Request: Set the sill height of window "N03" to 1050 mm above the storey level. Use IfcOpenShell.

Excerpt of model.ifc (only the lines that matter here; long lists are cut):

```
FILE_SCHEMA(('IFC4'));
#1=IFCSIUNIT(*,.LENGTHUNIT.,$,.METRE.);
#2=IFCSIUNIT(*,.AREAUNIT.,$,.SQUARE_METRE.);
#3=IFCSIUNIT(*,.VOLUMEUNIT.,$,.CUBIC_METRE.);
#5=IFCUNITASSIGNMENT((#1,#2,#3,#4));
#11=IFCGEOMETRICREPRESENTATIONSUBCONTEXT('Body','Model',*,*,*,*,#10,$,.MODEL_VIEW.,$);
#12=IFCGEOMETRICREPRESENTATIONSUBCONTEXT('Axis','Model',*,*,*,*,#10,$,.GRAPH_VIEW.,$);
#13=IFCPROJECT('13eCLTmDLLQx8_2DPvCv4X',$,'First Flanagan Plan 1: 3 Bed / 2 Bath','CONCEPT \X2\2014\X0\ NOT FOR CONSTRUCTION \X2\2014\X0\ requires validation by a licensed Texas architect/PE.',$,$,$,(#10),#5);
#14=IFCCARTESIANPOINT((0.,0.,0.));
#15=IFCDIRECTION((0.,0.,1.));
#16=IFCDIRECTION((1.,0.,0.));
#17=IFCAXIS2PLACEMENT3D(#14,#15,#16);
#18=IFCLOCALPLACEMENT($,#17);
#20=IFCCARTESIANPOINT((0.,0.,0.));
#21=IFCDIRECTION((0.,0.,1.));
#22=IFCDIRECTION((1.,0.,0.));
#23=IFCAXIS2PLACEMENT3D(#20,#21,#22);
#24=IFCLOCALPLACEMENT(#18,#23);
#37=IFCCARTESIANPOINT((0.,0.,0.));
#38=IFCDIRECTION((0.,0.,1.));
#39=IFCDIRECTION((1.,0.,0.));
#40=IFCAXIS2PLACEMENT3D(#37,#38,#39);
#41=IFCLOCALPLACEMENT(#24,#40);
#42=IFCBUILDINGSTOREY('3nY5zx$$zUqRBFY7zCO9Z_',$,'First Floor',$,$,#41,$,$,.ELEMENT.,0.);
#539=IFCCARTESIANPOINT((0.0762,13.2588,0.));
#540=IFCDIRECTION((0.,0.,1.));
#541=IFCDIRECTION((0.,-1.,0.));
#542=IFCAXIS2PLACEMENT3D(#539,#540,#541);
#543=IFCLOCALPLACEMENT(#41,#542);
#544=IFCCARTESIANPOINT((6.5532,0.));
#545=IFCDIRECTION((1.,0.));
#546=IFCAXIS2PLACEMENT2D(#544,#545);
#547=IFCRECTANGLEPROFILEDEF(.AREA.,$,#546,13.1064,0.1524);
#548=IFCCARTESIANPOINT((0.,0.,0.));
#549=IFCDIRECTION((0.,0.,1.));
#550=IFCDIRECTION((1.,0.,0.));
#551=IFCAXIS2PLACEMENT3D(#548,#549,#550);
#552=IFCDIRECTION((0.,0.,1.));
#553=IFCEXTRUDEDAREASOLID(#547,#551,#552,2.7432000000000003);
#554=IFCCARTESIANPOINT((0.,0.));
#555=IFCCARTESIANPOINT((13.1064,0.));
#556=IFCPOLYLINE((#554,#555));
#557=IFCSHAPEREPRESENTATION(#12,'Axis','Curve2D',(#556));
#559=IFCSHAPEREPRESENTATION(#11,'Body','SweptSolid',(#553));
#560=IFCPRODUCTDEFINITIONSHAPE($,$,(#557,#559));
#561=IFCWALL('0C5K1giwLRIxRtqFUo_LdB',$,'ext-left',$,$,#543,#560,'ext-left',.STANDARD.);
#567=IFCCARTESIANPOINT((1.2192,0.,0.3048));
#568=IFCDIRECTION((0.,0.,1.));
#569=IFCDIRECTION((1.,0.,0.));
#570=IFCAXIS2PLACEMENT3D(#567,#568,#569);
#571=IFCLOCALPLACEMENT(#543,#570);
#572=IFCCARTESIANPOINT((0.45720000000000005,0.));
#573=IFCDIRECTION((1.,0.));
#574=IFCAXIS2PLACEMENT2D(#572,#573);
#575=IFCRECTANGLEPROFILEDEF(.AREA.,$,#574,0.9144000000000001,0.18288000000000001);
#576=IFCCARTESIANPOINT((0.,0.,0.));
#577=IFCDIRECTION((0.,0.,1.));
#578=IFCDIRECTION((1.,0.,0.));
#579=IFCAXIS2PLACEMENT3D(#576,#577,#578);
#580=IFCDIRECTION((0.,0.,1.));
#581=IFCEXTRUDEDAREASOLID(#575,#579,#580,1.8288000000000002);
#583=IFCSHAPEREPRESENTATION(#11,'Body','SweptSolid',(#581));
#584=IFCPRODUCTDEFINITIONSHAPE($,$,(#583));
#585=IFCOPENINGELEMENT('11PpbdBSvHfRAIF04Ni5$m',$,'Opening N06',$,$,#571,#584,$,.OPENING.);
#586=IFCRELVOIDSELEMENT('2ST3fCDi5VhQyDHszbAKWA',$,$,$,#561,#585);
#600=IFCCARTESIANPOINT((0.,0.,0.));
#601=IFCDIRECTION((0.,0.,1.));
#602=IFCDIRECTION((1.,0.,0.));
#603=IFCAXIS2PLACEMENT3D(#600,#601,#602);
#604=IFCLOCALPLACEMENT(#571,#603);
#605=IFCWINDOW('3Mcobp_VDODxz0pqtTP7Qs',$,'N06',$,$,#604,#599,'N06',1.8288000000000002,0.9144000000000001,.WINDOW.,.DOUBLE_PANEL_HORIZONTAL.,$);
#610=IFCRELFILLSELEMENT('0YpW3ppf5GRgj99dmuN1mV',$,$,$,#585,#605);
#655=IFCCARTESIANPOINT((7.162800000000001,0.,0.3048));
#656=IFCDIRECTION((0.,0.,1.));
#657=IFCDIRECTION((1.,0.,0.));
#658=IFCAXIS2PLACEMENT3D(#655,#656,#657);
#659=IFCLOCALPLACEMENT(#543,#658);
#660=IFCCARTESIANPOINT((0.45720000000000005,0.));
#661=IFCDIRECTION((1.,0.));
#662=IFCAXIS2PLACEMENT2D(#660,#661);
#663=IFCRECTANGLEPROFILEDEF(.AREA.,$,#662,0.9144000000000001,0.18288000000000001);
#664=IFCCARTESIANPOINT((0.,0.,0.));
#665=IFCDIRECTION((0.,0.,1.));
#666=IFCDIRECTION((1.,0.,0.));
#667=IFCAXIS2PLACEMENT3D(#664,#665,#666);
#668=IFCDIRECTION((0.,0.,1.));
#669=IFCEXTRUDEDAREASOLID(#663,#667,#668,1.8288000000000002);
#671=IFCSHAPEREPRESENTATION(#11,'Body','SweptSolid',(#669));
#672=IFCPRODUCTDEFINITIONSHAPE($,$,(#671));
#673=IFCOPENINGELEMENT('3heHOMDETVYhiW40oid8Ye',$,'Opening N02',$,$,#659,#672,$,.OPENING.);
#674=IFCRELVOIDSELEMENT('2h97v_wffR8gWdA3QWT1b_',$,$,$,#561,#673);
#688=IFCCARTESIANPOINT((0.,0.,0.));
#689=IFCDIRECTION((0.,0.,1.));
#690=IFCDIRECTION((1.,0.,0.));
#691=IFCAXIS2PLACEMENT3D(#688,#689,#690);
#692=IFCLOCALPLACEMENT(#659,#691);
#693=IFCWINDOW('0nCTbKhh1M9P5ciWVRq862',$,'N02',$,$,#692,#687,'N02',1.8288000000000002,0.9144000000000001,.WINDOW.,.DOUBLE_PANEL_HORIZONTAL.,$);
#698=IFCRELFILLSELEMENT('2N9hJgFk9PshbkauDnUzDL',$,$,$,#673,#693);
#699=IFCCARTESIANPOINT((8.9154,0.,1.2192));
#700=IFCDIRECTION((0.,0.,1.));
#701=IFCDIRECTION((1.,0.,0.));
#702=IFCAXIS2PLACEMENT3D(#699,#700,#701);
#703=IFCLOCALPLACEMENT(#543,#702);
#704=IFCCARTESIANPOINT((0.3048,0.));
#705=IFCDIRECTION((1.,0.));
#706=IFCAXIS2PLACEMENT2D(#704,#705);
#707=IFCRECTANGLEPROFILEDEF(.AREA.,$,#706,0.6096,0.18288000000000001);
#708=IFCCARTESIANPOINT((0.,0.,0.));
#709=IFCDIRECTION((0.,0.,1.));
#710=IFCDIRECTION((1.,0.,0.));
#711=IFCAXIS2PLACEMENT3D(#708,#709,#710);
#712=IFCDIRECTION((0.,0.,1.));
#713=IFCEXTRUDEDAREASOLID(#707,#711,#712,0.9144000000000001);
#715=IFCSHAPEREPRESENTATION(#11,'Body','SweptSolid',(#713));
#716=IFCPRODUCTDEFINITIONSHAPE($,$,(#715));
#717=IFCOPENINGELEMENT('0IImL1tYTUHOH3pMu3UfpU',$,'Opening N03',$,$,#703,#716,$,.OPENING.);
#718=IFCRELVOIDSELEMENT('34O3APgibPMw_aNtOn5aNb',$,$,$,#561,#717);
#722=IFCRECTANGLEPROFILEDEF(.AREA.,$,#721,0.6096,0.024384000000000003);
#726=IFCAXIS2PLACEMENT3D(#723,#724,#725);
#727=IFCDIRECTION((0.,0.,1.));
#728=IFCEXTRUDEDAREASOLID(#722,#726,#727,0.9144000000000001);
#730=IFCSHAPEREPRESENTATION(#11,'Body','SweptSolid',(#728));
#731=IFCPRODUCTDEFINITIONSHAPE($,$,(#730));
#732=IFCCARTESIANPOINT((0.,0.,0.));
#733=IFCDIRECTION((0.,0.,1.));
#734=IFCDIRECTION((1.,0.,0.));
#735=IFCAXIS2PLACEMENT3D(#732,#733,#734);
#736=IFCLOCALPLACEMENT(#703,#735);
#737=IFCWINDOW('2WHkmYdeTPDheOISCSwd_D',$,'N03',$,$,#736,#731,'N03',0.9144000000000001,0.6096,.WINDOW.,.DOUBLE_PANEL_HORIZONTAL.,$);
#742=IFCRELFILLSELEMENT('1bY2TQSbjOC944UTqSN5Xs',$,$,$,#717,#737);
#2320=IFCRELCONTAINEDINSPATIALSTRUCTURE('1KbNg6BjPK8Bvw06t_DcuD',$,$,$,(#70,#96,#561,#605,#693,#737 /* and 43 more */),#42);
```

```python
import numpy as np
import ifcopenshell
import ifcopenshell.api.geometry
import ifcopenshell.geom
import ifcopenshell.util.element
import ifcopenshell.util.placement
import ifcopenshell.util.shape
import ifcopenshell.util.unit

model = ifcopenshell.open("model.ifc")
unit_scale = ifcopenshell.util.unit.calculate_unit_scale(model)

window = model.by_guid("2WHkmYdeTPDheOISCSwd_D")
opening = window.FillsVoids[0].RelatingOpeningElement
storey = ifcopenshell.util.element.get_container(window, ifc_class="IfcBuildingStorey")
level = ifcopenshell.util.placement.get_local_placement(storey.ObjectPlacement)[2, 3]

# The opening's origin need not be at the sill, so measure its lowest point.
shape = ifcopenshell.geom.create_shape(ifcopenshell.geom.settings(), opening)
bottom = ifcopenshell.util.shape.get_shape_bottom_elevation(shape, shape.geometry) / unit_scale
dz = level + 1.05 - bottom

shift = np.array([0.0, 0.0, dz])
# The window is placed relative to its opening, so it follows when the opening moves.
matrix = ifcopenshell.util.placement.get_local_placement(opening.ObjectPlacement)
matrix[:3, 3] += shift
ifcopenshell.api.geometry.edit_object_placement(
    model, product=opening, matrix=matrix, is_si=False, should_transform_children=True
)

print(f"moved by {dz * unit_scale:+.3f} m")

model.write("model_rev.ifc")
```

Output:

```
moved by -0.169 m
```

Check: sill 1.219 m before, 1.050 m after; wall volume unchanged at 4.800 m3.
